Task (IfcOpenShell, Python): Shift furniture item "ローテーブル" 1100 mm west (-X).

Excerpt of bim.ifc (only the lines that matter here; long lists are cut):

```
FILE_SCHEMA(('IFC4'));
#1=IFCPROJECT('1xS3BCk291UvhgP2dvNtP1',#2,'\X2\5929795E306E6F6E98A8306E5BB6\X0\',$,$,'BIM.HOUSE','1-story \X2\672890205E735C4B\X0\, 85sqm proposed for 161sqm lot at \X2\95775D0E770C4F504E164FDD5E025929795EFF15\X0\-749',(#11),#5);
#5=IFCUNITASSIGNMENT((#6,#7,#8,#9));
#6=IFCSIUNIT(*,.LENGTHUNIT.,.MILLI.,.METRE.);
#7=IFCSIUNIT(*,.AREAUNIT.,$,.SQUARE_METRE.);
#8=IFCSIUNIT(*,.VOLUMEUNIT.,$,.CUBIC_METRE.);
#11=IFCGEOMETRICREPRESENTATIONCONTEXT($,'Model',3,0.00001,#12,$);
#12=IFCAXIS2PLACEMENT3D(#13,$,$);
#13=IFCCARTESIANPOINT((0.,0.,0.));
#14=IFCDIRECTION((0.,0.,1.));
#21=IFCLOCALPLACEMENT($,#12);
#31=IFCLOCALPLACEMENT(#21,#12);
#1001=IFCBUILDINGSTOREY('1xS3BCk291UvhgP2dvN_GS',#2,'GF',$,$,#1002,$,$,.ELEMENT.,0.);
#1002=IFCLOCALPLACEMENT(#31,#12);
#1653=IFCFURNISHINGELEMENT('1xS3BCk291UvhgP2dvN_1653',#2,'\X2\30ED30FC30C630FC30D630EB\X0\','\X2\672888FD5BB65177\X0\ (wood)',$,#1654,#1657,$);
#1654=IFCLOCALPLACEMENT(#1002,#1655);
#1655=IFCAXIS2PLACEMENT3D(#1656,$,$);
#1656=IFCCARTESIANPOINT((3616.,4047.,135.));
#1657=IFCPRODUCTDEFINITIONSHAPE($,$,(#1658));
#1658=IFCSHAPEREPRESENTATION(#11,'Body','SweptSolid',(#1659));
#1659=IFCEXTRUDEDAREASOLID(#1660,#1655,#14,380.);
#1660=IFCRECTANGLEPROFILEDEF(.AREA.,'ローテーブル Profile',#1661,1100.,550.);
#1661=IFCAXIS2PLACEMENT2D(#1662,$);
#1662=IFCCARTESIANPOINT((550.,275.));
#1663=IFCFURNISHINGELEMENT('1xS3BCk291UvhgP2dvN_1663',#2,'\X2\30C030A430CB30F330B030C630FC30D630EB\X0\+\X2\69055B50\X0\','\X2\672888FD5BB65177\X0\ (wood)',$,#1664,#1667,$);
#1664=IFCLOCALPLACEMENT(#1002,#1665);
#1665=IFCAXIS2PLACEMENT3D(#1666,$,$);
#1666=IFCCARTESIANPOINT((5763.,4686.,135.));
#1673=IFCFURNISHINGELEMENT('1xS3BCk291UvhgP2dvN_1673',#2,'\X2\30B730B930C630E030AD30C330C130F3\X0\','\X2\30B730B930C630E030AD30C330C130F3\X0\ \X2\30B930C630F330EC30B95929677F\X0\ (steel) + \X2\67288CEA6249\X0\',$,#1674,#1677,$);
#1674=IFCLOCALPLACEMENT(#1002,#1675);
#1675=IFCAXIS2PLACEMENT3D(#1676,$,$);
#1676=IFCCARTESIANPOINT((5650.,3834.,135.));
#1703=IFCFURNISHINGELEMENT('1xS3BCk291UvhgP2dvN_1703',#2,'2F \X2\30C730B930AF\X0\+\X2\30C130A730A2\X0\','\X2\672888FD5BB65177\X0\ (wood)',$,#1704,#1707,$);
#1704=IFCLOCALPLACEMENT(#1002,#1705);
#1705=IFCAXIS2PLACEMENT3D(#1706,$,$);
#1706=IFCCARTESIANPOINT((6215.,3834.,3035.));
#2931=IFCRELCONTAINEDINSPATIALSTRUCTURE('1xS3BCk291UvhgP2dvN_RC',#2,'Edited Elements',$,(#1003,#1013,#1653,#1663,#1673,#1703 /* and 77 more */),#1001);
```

```python
import ifcopenshell
import ifcopenshell.api.geometry
import ifcopenshell.util.placement

model = ifcopenshell.open("bim.ifc")

item = model.by_guid("1xS3BCk291UvhgP2dvN_1653")
matrix = ifcopenshell.util.placement.get_local_placement(item.ObjectPlacement)
matrix[0, 3] -= 1100.0
ifcopenshell.api.geometry.edit_object_placement(model, product=item, matrix=matrix, is_si=False)

print(ifcopenshell.util.placement.get_local_placement(item.ObjectPlacement).round(3) + 0.0)

model.write("bim_updated.ifc")
```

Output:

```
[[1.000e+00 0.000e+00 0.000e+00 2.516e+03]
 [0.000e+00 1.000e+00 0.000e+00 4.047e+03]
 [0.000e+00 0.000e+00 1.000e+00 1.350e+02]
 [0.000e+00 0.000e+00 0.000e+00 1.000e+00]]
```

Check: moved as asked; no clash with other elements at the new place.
